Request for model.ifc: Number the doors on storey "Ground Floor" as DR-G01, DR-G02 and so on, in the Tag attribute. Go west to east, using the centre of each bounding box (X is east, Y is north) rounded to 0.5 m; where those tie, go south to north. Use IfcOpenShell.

First a look at what the model holds.

```python
import ifcopenshell
import ifcopenshell.util.element
import ifcopenshell.util.placement

model = ifcopenshell.open("model.ifc")
print(model.schema)
storey = next(s for s in model.by_type("IfcBuildingStorey") if s.Name == "Ground Floor")
doors = [e for e in ifcopenshell.util.element.get_decomposition(storey) if e.is_a("IfcDoor")]
for e in sorted(doors, key=lambda e: e.id()):
    origin = ifcopenshell.util.placement.get_local_placement(e.ObjectPlacement)[:3, 3]
    print(e.id(), e.Tag, e.Name, origin.round(2) + 0.0, sep=" | ")
```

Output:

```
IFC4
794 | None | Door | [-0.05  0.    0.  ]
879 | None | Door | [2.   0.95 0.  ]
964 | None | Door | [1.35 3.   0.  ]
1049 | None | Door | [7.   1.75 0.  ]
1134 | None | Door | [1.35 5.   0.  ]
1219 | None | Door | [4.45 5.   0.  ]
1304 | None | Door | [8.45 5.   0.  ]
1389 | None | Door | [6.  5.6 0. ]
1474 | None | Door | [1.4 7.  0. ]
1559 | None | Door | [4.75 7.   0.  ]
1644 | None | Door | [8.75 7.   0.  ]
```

```python
import ifcopenshell
import ifcopenshell.geom
import ifcopenshell.util.element
import ifcopenshell.util.shape

model = ifcopenshell.open("model.ifc")
settings = ifcopenshell.geom.settings()
settings.set("use-world-coords", True)


def centre(element):
    shape = ifcopenshell.geom.create_shape(settings, element)
    return ifcopenshell.util.shape.get_bbox_centroid(shape.geometry)


storey = next(s for s in model.by_type("IfcBuildingStorey") if s.Name == "Ground Floor")
doors = [e for e in ifcopenshell.util.element.get_decomposition(storey) if e.is_a("IfcDoor")]

# Insertion points can sit at a corner or the storey origin, so sort by the geometry (in metres).
centres = {e: centre(e) for e in doors}
doors.sort(key=lambda e: (round(centres[e][0] / 0.5), centres[e][1]))

for i, e in enumerate(doors, start=1):
    number = f"DR-G{i:02d}"
    e.Tag = number
    print(e.id(), number)

model.write("model_edited.ifc")
```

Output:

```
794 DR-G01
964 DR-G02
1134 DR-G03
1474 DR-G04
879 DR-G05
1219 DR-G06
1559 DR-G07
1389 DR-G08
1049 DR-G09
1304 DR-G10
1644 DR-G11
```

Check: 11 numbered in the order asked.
